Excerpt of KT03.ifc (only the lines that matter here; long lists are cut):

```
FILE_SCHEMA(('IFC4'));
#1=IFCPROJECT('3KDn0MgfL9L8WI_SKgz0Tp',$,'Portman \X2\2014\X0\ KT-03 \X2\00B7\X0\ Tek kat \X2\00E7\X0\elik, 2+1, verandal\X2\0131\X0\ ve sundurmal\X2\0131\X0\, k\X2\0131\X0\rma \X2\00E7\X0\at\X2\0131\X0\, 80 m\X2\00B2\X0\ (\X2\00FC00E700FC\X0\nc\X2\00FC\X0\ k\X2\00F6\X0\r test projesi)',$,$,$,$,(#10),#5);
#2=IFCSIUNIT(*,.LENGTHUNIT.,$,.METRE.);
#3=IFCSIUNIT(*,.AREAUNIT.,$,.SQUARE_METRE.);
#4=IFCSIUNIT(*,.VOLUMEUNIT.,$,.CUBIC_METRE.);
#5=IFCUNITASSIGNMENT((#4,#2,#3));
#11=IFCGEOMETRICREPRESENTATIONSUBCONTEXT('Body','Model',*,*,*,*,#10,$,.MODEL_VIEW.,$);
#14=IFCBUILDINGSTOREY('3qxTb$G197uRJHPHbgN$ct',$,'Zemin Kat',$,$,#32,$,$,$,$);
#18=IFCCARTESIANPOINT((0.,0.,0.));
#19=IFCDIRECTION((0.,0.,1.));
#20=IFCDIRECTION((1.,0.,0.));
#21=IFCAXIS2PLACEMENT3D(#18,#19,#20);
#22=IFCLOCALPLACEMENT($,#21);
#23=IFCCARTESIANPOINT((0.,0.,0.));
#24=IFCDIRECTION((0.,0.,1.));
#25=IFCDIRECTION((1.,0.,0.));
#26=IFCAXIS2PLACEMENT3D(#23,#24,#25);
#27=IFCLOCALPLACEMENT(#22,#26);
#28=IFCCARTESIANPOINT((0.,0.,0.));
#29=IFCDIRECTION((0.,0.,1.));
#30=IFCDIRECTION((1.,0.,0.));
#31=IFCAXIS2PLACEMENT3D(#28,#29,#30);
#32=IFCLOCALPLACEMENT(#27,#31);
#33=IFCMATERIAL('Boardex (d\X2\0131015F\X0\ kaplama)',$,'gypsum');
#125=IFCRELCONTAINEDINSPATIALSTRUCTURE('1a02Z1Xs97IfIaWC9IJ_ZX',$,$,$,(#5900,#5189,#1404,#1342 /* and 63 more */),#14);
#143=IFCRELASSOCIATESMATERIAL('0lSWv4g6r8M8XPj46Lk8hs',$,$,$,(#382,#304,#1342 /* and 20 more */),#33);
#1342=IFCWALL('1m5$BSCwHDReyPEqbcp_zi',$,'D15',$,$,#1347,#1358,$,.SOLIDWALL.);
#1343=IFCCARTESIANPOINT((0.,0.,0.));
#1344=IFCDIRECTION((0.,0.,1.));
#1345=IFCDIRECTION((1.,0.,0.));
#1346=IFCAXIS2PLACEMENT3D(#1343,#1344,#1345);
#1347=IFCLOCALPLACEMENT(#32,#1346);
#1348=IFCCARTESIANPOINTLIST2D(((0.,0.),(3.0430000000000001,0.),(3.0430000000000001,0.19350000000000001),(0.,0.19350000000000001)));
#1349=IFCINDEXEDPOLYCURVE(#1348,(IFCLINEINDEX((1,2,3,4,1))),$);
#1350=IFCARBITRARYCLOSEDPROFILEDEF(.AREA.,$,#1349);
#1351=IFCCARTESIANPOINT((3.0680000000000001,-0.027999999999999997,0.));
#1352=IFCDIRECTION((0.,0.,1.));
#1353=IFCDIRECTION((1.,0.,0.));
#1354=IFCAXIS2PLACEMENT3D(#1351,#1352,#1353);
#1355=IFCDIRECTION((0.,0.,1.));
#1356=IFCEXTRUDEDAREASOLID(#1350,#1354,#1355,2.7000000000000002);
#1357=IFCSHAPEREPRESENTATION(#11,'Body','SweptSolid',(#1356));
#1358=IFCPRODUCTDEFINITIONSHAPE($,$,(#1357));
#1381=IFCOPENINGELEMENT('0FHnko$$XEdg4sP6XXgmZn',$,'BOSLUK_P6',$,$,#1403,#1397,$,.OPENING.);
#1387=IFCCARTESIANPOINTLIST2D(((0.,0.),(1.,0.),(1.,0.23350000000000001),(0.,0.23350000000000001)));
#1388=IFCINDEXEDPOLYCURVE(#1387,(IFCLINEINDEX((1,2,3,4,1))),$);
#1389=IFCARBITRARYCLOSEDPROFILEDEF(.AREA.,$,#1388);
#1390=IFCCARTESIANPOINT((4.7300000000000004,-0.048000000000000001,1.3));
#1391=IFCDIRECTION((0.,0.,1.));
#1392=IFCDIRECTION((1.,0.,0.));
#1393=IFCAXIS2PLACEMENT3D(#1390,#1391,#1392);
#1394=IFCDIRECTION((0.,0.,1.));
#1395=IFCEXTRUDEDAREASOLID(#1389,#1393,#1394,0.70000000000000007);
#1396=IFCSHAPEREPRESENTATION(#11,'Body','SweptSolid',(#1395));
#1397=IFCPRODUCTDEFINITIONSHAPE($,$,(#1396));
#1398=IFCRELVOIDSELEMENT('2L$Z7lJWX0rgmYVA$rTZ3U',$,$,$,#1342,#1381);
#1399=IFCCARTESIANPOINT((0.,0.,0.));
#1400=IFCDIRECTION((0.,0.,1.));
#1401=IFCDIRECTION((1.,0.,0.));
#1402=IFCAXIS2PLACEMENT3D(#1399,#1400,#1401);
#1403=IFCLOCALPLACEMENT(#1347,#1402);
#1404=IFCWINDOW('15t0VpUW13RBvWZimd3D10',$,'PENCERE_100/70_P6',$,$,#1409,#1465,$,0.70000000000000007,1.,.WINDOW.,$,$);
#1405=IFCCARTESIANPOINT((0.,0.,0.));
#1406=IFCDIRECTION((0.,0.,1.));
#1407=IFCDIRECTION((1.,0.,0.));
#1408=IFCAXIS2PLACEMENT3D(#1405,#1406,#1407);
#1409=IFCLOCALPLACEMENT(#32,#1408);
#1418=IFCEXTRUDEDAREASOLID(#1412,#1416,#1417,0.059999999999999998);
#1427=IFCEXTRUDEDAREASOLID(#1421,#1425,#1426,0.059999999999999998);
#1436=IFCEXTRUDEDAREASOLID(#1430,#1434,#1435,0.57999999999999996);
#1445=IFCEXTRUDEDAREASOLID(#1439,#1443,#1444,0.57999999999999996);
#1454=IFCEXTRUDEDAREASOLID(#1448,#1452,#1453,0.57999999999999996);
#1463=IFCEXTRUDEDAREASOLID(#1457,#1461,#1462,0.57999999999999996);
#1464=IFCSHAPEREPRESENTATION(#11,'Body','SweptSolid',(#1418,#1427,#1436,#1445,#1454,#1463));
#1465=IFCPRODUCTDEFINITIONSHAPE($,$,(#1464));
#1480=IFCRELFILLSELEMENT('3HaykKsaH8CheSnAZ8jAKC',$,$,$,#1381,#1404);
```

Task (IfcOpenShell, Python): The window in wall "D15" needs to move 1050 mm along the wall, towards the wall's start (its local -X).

```python
import ifcopenshell
import ifcopenshell.api.geometry
import ifcopenshell.util.placement
import ifcopenshell.util.unit

model = ifcopenshell.open("KT03.ifc")
unit_scale = ifcopenshell.util.unit.calculate_unit_scale(model)

window = model.by_id(1404)
opening = window.FillsVoids[0].RelatingOpeningElement
wall = opening.VoidsElements[0].RelatingBuildingElement

wall_matrix = ifcopenshell.util.placement.get_local_placement(wall.ObjectPlacement)
shift = wall_matrix[:3, 0] * -1.05 / unit_scale
before = ifcopenshell.util.placement.get_local_placement(window.ObjectPlacement)[:3, 3].copy()

# The window is not placed relative to its opening, so move both.
for product in (opening, window):
    matrix = ifcopenshell.util.placement.get_local_placement(product.ObjectPlacement)
    matrix[:3, 3] += shift
    ifcopenshell.api.geometry.edit_object_placement(model, product=product, matrix=matrix, is_si=False)

after = ifcopenshell.util.placement.get_local_placement(window.ObjectPlacement)[:3, 3]
print("window moved by", (after - before).round(3) + 0.0)

model.write("KT03_rev.ifc")
```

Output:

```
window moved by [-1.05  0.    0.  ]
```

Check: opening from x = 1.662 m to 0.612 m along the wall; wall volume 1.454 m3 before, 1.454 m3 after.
